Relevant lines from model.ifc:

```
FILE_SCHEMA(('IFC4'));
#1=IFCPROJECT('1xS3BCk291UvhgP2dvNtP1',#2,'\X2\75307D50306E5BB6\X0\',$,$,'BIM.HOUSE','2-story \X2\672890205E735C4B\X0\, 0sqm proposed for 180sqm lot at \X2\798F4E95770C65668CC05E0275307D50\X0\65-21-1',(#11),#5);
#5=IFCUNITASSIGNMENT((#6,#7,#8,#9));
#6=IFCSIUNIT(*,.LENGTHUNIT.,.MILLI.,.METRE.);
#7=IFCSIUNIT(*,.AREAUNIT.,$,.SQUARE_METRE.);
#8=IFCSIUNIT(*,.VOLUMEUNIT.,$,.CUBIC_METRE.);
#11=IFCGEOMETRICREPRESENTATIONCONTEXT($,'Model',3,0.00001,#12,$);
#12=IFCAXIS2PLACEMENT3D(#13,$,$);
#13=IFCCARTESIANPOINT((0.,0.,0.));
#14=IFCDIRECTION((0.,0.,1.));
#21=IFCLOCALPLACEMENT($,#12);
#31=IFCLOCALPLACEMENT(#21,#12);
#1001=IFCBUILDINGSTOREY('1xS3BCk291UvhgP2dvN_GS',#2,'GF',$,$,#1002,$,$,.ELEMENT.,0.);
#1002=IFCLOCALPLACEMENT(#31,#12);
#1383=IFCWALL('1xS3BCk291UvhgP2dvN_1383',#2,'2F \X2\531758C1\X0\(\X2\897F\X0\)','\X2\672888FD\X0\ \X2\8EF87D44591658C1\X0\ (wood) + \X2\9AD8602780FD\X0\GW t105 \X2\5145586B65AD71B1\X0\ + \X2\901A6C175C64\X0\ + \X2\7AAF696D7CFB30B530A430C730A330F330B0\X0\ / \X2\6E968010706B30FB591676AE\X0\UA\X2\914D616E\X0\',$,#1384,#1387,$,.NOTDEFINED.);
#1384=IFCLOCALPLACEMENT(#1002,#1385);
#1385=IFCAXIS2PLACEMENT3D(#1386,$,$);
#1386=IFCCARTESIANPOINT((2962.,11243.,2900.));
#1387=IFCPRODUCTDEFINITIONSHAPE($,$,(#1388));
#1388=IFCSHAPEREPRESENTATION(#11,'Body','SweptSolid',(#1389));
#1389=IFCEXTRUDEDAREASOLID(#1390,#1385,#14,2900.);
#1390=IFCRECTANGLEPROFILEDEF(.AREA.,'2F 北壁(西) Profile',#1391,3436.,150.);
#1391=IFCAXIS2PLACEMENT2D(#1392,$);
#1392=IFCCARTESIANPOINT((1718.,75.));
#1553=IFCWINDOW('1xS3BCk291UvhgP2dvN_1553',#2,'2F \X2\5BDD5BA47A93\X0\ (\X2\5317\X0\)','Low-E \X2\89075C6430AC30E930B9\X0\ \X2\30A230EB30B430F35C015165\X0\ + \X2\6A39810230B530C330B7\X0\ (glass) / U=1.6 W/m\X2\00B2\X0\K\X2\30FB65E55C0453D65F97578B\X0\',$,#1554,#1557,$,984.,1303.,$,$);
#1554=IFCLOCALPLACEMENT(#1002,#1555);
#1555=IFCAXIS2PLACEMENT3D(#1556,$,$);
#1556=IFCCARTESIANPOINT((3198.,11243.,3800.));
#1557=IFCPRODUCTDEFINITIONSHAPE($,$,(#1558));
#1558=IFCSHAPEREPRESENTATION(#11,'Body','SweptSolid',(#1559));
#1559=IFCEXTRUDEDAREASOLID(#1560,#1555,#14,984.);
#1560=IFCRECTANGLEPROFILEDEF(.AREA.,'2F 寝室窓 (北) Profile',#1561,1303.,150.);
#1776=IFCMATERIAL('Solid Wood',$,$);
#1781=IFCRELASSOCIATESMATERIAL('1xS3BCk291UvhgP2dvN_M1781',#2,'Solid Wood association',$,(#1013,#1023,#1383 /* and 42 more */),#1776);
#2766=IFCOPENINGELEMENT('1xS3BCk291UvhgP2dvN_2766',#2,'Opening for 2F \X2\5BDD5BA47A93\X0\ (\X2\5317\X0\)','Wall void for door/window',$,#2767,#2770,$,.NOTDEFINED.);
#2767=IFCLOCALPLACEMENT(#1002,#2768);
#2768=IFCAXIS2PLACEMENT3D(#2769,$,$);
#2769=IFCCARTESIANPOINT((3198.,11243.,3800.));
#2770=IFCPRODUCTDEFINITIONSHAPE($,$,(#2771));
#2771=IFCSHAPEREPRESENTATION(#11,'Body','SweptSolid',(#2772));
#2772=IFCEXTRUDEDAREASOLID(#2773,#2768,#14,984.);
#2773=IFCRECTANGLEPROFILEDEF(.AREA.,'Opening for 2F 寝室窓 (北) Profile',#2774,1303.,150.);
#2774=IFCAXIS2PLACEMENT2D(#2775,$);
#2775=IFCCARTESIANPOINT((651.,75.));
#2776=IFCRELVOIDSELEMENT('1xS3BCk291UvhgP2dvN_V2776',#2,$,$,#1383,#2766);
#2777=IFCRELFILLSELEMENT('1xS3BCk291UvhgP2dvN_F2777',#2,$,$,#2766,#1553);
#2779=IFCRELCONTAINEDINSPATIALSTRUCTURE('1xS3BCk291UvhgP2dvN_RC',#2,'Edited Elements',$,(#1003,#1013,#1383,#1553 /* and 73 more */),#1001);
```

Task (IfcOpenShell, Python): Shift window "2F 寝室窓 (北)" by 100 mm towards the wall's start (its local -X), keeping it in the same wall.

```python
import ifcopenshell
import ifcopenshell.api.geometry
import ifcopenshell.util.placement
import ifcopenshell.util.unit

model = ifcopenshell.open("model.ifc")
unit_scale = ifcopenshell.util.unit.calculate_unit_scale(model)

window = model.by_guid("1xS3BCk291UvhgP2dvN_1553")
opening = window.FillsVoids[0].RelatingOpeningElement
wall = opening.VoidsElements[0].RelatingBuildingElement

wall_matrix = ifcopenshell.util.placement.get_local_placement(wall.ObjectPlacement)
shift = wall_matrix[:3, 0] * -0.1 / unit_scale
before = ifcopenshell.util.placement.get_local_placement(window.ObjectPlacement)[:3, 3].copy()

# The window is not placed relative to its opening, so move both.
for product in (opening, window):
    matrix = ifcopenshell.util.placement.get_local_placement(product.ObjectPlacement)
    matrix[:3, 3] += shift
    ifcopenshell.api.geometry.edit_object_placement(model, product=product, matrix=matrix, is_si=False)

after = ifcopenshell.util.placement.get_local_placement(window.ObjectPlacement)[:3, 3]
print("window moved by", (after - before).round(3) + 0.0)

model.write("model_v2.ifc")
```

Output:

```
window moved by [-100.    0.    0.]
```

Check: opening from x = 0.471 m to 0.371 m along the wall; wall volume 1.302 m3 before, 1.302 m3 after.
